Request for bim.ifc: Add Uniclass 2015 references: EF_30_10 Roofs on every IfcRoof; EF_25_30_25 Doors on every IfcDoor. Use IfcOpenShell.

First a look at what the model holds.

```python
import ifcopenshell

model = ifcopenshell.open("bim.ifc")
print(model.schema)
print("classifications:", [c.Name for c in model.by_type("IfcClassification")])
for ifc_class in ("IfcDoor", "IfcRoof", "IfcStair", "IfcWall", "IfcWindow"):
    print(ifc_class, len(model.by_type(ifc_class)))
```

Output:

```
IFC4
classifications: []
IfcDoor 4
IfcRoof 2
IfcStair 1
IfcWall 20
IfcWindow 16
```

```python
import ifcopenshell
import ifcopenshell.api.classification

model = ifcopenshell.open("bim.ifc")

system = ifcopenshell.api.classification.add_classification(model, classification="Uniclass 2015")

codes = {
    "IfcRoof": ("EF_30_10", "Roofs"),
    "IfcDoor": ("EF_25_30_25", "Doors"),
}
for ifc_class, (code, name) in codes.items():
    products = model.by_type(ifc_class)
    ifcopenshell.api.classification.add_reference(
        model, products=products, classification=system, identification=code, name=name
    )
    print(code, len(products))

model.write("bim-out.ifc")
```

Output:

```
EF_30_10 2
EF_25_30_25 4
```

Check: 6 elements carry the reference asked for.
